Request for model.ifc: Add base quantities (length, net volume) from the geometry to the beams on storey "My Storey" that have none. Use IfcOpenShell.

First a look at what the model holds.

```python
import ifcopenshell
import ifcopenshell.util.element
import ifcopenshell.util.unit

model = ifcopenshell.open("model.ifc")
print(model.schema)
for unit_type in ("LENGTHUNIT", "AREAUNIT", "VOLUMEUNIT"):
    print(unit_type, ifcopenshell.util.unit.calculate_unit_scale(model, unit_type))
storey = next(s for s in model.by_type("IfcBuildingStorey") if s.Name == "My Storey")
beams = [e for e in ifcopenshell.util.element.get_decomposition(storey) if e.is_a("IfcBeam")]
for e in sorted(beams, key=lambda e: e.id()):
    print(e.id(), e.is_a(), e.Name, list(ifcopenshell.util.element.get_psets(e, qtos_only=True)), sep=" | ")
```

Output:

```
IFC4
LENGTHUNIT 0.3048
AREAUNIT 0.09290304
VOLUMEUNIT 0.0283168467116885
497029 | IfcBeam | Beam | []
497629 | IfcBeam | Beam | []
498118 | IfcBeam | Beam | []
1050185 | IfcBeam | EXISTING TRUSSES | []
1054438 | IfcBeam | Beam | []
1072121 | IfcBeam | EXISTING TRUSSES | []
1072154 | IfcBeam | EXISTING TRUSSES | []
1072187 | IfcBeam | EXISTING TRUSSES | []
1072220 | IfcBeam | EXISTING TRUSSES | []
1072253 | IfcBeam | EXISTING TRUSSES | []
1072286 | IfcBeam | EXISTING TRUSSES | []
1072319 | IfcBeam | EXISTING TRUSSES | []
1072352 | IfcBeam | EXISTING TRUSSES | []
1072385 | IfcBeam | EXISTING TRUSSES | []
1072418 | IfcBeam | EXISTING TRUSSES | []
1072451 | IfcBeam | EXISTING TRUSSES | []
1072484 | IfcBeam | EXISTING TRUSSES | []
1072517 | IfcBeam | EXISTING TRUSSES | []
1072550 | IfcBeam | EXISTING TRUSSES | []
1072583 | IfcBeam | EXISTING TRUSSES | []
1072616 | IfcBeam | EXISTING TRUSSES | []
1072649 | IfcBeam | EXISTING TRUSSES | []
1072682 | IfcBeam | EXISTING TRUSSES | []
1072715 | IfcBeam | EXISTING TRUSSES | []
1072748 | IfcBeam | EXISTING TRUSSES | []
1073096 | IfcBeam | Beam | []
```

```python
import ifcopenshell
import ifcopenshell.api.pset
import ifcopenshell.geom
import ifcopenshell.util.element
import ifcopenshell.util.shape
import ifcopenshell.util.unit

model = ifcopenshell.open("model.ifc")
unit_scale = ifcopenshell.util.unit.calculate_unit_scale(model)
volume_scale = ifcopenshell.util.unit.calculate_unit_scale(model, "VOLUMEUNIT")
settings = ifcopenshell.geom.settings()

storey = next(s for s in model.by_type("IfcBuildingStorey") if s.Name == "My Storey")
beams = [e for e in ifcopenshell.util.element.get_decomposition(storey) if e.is_a("IfcBeam")]

for e in sorted(beams, key=lambda e: e.id()):
    if ifcopenshell.util.element.get_psets(e, qtos_only=True, should_inherit=False):
        continue
    # Geometry comes back in metres, in the element's own axes.
    shape = ifcopenshell.geom.create_shape(settings, e)
    values = {
        "Length": ifcopenshell.util.shape.get_max_xyz(shape.geometry) / unit_scale,
        "NetVolume": ifcopenshell.util.shape.get_volume(shape.geometry) / volume_scale,
    }
    qto = ifcopenshell.api.pset.add_qto(model, product=e, name="Qto_BeamBaseQuantities")
    ifcopenshell.api.pset.edit_qto(model, qto=qto, properties=values)
    print(e.id(), {k: round(v, 3) for k, v in values.items()})

model.write("model-out.ifc")
```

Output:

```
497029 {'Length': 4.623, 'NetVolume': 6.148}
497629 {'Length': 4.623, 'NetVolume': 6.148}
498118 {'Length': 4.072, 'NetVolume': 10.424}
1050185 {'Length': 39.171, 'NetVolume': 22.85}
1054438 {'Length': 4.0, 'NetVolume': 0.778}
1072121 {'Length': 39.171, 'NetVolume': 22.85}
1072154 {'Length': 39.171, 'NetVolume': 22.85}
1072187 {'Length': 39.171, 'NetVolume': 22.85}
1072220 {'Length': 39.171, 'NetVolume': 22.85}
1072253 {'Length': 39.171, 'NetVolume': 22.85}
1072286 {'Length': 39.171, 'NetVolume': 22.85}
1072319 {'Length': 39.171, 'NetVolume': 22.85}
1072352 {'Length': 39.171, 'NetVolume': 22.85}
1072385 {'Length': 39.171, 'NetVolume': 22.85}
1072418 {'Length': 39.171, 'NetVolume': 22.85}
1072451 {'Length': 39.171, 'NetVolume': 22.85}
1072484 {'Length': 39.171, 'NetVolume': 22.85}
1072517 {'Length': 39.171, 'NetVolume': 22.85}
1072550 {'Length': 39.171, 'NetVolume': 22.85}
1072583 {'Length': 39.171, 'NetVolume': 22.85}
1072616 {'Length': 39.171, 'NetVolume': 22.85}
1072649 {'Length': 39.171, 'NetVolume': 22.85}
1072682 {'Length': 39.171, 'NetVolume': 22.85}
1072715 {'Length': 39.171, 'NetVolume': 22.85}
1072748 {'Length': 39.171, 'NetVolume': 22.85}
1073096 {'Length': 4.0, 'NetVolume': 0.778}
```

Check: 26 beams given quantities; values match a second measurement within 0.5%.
